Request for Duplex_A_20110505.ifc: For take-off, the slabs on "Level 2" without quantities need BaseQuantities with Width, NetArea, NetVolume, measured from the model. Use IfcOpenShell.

First a look at what the model holds.

```python
import ifcopenshell
import ifcopenshell.util.element
import ifcopenshell.util.unit

model = ifcopenshell.open("Duplex_A_20110505.ifc")
print(model.schema)
for unit_type in ("LENGTHUNIT", "AREAUNIT", "VOLUMEUNIT"):
    print(unit_type, ifcopenshell.util.unit.calculate_unit_scale(model, unit_type))
storey = next(s for s in model.by_type("IfcBuildingStorey") if s.Name == "Level 2")
slabs = [e for e in ifcopenshell.util.element.get_decomposition(storey) if e.is_a("IfcSlab")]
for e in sorted(slabs, key=lambda e: e.id()):
    print(e.id(), e.is_a(), e.Name, list(ifcopenshell.util.element.get_psets(e, qtos_only=True)), sep=" | ")
```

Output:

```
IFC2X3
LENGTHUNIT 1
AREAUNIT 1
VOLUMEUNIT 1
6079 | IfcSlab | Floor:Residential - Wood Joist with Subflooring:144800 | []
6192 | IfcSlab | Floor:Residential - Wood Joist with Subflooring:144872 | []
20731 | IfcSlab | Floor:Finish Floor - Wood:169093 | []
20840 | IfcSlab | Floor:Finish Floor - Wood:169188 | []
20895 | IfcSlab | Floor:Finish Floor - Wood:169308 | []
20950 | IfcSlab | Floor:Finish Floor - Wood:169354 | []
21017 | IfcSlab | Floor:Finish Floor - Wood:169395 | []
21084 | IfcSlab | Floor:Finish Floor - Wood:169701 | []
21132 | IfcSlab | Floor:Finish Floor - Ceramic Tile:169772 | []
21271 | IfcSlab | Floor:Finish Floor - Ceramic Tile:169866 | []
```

```python
import ifcopenshell
import ifcopenshell.api.pset
import ifcopenshell.geom
import ifcopenshell.util.element
import ifcopenshell.util.shape
import ifcopenshell.util.unit

model = ifcopenshell.open("Duplex_A_20110505.ifc")
unit_scale = ifcopenshell.util.unit.calculate_unit_scale(model)
area_scale = ifcopenshell.util.unit.calculate_unit_scale(model, "AREAUNIT")
volume_scale = ifcopenshell.util.unit.calculate_unit_scale(model, "VOLUMEUNIT")
settings = ifcopenshell.geom.settings()

storey = next(s for s in model.by_type("IfcBuildingStorey") if s.Name == "Level 2")
slabs = [e for e in ifcopenshell.util.element.get_decomposition(storey) if e.is_a("IfcSlab")]

for e in sorted(slabs, key=lambda e: e.id()):
    if ifcopenshell.util.element.get_psets(e, qtos_only=True, should_inherit=False):
        continue
    # Geometry comes back in metres, in the element's own axes.
    shape = ifcopenshell.geom.create_shape(settings, e)
    values = {
        "Width": ifcopenshell.util.shape.get_z(shape.geometry) / unit_scale,
        "NetArea": ifcopenshell.util.shape.get_footprint_area(shape.geometry) / area_scale,
        "NetVolume": ifcopenshell.util.shape.get_volume(shape.geometry) / volume_scale,
    }
    qto = ifcopenshell.api.pset.add_qto(model, product=e, name="BaseQuantities")
    ifcopenshell.api.pset.edit_qto(model, qto=qto, properties=values)
    print(e.id(), {k: round(v, 3) for k, v in values.items()})

model.write("Duplex_A_20110505-out.ifc")
```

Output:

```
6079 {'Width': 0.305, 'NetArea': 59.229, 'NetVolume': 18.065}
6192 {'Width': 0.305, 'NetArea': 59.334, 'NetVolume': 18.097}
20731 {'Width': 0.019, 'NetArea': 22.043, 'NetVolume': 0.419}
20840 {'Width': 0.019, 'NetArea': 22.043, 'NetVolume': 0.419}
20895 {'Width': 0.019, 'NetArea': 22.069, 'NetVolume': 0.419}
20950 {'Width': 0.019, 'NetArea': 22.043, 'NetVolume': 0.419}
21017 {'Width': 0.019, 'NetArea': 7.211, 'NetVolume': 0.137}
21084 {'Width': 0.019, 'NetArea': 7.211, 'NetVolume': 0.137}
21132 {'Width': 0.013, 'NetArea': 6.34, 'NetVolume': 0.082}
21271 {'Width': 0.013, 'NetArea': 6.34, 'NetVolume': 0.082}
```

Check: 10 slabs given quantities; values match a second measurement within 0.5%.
